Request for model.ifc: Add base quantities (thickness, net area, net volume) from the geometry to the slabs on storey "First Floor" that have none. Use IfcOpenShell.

First a look at what the model holds.

```python
import ifcopenshell
import ifcopenshell.util.element
import ifcopenshell.util.unit

model = ifcopenshell.open("model.ifc")
print(model.schema)
for unit_type in ("LENGTHUNIT", "AREAUNIT", "VOLUMEUNIT"):
    print(unit_type, ifcopenshell.util.unit.calculate_unit_scale(model, unit_type))
storey = next(s for s in model.by_type("IfcBuildingStorey") if s.Name == "First Floor")
slabs = [e for e in ifcopenshell.util.element.get_decomposition(storey) if e.is_a("IfcSlab")]
for e in sorted(slabs, key=lambda e: e.id()):
    print(e.id(), e.is_a(), e.Name, list(ifcopenshell.util.element.get_psets(e, qtos_only=True)), sep=" | ")
```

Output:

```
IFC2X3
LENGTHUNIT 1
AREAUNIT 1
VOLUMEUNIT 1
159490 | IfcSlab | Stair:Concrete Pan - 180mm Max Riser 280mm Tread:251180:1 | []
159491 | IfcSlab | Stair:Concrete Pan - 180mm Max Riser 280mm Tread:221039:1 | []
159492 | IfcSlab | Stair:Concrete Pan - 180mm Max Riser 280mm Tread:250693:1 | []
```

```python
import ifcopenshell
import ifcopenshell.api.pset
import ifcopenshell.geom
import ifcopenshell.util.element
import ifcopenshell.util.shape
import ifcopenshell.util.unit

model = ifcopenshell.open("model.ifc")
unit_scale = ifcopenshell.util.unit.calculate_unit_scale(model)
area_scale = ifcopenshell.util.unit.calculate_unit_scale(model, "AREAUNIT")
volume_scale = ifcopenshell.util.unit.calculate_unit_scale(model, "VOLUMEUNIT")
settings = ifcopenshell.geom.settings()

storey = next(s for s in model.by_type("IfcBuildingStorey") if s.Name == "First Floor")
slabs = [e for e in ifcopenshell.util.element.get_decomposition(storey) if e.is_a("IfcSlab")]

for e in sorted(slabs, key=lambda e: e.id()):
    if ifcopenshell.util.element.get_psets(e, qtos_only=True, should_inherit=False):
        continue
    # Geometry comes back in metres, in the element's own axes.
    shape = ifcopenshell.geom.create_shape(settings, e)
    values = {
        "Width": ifcopenshell.util.shape.get_z(shape.geometry) / unit_scale,
        "NetArea": ifcopenshell.util.shape.get_footprint_area(shape.geometry) / area_scale,
        "NetVolume": ifcopenshell.util.shape.get_volume(shape.geometry) / volume_scale,
    }
    qto = ifcopenshell.api.pset.add_qto(model, product=e, name="BaseQuantities")
    ifcopenshell.api.pset.edit_qto(model, qto=qto, properties=values)
    print(e.id(), {k: round(v, 3) for k, v in values.items()})

model.write("model_updated.ifc")
```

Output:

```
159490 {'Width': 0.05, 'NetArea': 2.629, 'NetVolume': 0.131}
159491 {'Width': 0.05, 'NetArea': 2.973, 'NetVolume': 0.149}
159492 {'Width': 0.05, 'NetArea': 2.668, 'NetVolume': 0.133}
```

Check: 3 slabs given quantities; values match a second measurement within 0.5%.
